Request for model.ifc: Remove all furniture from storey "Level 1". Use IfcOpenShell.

First a look at what the model holds.

```python
import ifcopenshell
import ifcopenshell.util.element

model = ifcopenshell.open("model.ifc")
print(model.schema)
storey = next(s for s in model.by_type("IfcBuildingStorey") if s.Name == "Level 1")
furniture = [e for e in ifcopenshell.util.element.get_decomposition(storey) if e.is_a("IfcFurnishingElement")]
seen = {}
for e in furniture:
    element_type = ifcopenshell.util.element.get_type(e)
    name = element_type.Name if element_type not in (None, e) else None
    seen[name] = seen.get(name, 0) + 1
for name, count in sorted(seen.items(), key=str):
    print(count, "x", name)
```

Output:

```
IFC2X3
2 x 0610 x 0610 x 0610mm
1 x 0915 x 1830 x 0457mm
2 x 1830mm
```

```python
import ifcopenshell
import ifcopenshell.api.root
import ifcopenshell.util.element

model = ifcopenshell.open("model.ifc")

storey = next(s for s in model.by_type("IfcBuildingStorey") if s.Name == "Level 1")
furniture = [e for e in ifcopenshell.util.element.get_decomposition(storey) if e.is_a("IfcFurnishingElement")]

for e in furniture:
    ifcopenshell.api.root.remove_product(model, product=e)
print(len(furniture), "removed")

model.write("model_rev.ifc")
```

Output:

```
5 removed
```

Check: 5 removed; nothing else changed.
